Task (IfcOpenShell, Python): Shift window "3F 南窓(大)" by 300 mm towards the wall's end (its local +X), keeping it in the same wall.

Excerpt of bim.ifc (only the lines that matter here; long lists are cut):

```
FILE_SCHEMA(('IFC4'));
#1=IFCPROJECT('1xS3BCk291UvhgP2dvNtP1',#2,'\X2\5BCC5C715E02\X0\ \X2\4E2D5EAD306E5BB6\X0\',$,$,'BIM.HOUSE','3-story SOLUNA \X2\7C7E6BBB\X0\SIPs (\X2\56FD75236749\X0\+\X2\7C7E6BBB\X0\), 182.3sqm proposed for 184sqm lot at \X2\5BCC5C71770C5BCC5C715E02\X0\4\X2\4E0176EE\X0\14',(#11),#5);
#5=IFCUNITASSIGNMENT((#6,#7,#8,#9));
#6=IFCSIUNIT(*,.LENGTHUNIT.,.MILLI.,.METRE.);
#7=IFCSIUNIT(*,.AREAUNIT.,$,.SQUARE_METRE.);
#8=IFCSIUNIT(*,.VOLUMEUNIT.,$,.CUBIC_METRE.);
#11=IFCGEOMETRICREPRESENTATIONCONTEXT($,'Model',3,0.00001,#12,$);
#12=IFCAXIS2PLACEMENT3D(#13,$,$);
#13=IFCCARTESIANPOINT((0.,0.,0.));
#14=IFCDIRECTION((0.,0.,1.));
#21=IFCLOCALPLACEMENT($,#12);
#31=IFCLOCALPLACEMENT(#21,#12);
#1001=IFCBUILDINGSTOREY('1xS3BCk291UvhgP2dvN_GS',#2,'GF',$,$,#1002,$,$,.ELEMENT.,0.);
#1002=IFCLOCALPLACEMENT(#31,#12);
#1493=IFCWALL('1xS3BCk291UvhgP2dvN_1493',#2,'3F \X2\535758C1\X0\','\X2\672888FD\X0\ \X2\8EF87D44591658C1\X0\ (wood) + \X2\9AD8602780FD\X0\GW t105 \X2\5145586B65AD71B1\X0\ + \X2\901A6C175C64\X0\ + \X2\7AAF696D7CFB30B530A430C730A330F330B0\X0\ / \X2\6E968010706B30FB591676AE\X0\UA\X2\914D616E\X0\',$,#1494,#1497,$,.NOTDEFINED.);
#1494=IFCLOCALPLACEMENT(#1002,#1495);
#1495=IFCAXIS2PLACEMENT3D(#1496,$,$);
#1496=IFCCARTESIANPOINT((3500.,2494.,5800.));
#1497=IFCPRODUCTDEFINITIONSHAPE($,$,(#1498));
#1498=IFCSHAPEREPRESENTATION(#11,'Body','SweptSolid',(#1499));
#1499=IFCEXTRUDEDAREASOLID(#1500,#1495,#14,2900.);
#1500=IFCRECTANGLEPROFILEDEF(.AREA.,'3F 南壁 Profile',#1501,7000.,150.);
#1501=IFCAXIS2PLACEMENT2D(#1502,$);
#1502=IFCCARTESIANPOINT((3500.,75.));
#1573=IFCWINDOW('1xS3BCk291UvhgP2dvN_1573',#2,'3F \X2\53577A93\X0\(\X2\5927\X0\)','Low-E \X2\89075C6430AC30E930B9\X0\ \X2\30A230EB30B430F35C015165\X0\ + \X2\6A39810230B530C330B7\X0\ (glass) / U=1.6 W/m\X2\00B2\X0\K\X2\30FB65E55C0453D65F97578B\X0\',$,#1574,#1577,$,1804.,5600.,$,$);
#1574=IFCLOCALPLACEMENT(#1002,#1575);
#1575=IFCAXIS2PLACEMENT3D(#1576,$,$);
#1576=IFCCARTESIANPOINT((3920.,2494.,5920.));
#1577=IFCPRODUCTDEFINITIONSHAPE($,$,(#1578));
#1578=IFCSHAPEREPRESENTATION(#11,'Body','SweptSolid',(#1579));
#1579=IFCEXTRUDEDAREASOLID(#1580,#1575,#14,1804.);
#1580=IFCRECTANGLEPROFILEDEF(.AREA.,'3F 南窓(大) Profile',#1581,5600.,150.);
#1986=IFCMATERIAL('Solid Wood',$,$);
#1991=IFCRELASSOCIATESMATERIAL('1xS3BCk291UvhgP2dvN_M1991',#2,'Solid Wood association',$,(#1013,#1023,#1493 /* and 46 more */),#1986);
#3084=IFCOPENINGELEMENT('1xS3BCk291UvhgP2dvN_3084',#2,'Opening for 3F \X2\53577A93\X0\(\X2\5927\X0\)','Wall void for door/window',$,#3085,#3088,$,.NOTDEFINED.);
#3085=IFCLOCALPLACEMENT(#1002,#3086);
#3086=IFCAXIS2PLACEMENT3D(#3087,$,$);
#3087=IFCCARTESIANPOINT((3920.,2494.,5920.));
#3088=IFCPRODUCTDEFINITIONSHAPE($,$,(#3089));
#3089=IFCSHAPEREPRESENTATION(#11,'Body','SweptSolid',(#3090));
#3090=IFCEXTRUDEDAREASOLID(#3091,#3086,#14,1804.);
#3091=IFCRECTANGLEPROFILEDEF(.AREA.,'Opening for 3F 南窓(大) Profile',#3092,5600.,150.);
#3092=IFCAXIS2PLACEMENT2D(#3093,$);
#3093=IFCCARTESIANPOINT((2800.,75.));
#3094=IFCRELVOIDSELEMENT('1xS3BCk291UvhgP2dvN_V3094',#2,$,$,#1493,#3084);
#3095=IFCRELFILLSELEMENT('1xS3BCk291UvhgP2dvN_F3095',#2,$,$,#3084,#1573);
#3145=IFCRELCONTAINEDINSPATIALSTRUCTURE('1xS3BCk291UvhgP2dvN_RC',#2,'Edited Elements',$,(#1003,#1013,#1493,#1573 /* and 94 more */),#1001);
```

```python
import ifcopenshell
import ifcopenshell.api.geometry
import ifcopenshell.util.placement
import ifcopenshell.util.unit

model = ifcopenshell.open("bim.ifc")
unit_scale = ifcopenshell.util.unit.calculate_unit_scale(model)

window = model.by_id(1573)
opening = window.FillsVoids[0].RelatingOpeningElement
wall = opening.VoidsElements[0].RelatingBuildingElement

wall_matrix = ifcopenshell.util.placement.get_local_placement(wall.ObjectPlacement)
shift = wall_matrix[:3, 0] * 0.3 / unit_scale
before = ifcopenshell.util.placement.get_local_placement(window.ObjectPlacement)[:3, 3].copy()

# The window is not placed relative to its opening, so move both.
for product in (opening, window):
    matrix = ifcopenshell.util.placement.get_local_placement(product.ObjectPlacement)
    matrix[:3, 3] += shift
    ifcopenshell.api.geometry.edit_object_placement(model, product=product, matrix=matrix, is_si=False)

after = ifcopenshell.util.placement.get_local_placement(window.ObjectPlacement)[:3, 3]
print("window moved by", (after - before).round(3) + 0.0)

model.write("bim_updated.ifc")
```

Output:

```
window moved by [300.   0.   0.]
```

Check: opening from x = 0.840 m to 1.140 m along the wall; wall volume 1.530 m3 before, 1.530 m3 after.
